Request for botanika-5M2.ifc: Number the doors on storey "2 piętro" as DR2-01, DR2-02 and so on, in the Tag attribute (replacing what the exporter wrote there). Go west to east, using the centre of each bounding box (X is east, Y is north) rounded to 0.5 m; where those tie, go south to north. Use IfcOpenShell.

First a look at what the model holds.

```python
import ifcopenshell
import ifcopenshell.util.element
import ifcopenshell.util.placement

model = ifcopenshell.open("botanika-5M2.ifc")
print(model.schema)
storey = next(s for s in model.by_type("IfcBuildingStorey") if s.Name == "2 piętro")
doors = [e for e in ifcopenshell.util.element.get_decomposition(storey) if e.is_a("IfcDoor")]
for e in sorted(doors, key=lambda e: e.id()):
    origin = ifcopenshell.util.placement.get_local_placement(e.ObjectPlacement)[:3, 3]
    print(e.id(), e.Tag, e.Name, origin.round(2) + 0.0, sep=" | ")
```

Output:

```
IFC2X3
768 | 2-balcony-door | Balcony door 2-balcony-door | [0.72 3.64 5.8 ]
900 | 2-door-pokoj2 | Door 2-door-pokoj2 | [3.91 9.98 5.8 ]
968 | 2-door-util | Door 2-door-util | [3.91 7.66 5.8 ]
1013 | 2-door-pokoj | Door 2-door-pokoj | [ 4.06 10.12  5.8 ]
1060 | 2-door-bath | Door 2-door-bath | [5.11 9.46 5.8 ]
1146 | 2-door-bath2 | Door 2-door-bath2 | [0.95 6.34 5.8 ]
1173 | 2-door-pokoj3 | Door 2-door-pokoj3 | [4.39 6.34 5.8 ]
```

```python
import ifcopenshell
import ifcopenshell.geom
import ifcopenshell.util.element
import ifcopenshell.util.shape

model = ifcopenshell.open("botanika-5M2.ifc")
settings = ifcopenshell.geom.settings()
settings.set("use-world-coords", True)


def centre(element):
    shape = ifcopenshell.geom.create_shape(settings, element)
    return ifcopenshell.util.shape.get_bbox_centroid(shape.geometry)


storey = next(s for s in model.by_type("IfcBuildingStorey") if s.Name == "2 piętro")
doors = [e for e in ifcopenshell.util.element.get_decomposition(storey) if e.is_a("IfcDoor")]

# Insertion points can sit at a corner or the storey origin, so sort by the geometry (in metres).
centres = {e: centre(e) for e in doors}
doors.sort(key=lambda e: (round(centres[e][0] / 0.5), centres[e][1]))

for i, e in enumerate(doors, start=1):
    number = f"DR2-{i:02d}"
    e.Tag = number
    print(e.id(), number)

model.write("botanika-5M2-out.ifc")
```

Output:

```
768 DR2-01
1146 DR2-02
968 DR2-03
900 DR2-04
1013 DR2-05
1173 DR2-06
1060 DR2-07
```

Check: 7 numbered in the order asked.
